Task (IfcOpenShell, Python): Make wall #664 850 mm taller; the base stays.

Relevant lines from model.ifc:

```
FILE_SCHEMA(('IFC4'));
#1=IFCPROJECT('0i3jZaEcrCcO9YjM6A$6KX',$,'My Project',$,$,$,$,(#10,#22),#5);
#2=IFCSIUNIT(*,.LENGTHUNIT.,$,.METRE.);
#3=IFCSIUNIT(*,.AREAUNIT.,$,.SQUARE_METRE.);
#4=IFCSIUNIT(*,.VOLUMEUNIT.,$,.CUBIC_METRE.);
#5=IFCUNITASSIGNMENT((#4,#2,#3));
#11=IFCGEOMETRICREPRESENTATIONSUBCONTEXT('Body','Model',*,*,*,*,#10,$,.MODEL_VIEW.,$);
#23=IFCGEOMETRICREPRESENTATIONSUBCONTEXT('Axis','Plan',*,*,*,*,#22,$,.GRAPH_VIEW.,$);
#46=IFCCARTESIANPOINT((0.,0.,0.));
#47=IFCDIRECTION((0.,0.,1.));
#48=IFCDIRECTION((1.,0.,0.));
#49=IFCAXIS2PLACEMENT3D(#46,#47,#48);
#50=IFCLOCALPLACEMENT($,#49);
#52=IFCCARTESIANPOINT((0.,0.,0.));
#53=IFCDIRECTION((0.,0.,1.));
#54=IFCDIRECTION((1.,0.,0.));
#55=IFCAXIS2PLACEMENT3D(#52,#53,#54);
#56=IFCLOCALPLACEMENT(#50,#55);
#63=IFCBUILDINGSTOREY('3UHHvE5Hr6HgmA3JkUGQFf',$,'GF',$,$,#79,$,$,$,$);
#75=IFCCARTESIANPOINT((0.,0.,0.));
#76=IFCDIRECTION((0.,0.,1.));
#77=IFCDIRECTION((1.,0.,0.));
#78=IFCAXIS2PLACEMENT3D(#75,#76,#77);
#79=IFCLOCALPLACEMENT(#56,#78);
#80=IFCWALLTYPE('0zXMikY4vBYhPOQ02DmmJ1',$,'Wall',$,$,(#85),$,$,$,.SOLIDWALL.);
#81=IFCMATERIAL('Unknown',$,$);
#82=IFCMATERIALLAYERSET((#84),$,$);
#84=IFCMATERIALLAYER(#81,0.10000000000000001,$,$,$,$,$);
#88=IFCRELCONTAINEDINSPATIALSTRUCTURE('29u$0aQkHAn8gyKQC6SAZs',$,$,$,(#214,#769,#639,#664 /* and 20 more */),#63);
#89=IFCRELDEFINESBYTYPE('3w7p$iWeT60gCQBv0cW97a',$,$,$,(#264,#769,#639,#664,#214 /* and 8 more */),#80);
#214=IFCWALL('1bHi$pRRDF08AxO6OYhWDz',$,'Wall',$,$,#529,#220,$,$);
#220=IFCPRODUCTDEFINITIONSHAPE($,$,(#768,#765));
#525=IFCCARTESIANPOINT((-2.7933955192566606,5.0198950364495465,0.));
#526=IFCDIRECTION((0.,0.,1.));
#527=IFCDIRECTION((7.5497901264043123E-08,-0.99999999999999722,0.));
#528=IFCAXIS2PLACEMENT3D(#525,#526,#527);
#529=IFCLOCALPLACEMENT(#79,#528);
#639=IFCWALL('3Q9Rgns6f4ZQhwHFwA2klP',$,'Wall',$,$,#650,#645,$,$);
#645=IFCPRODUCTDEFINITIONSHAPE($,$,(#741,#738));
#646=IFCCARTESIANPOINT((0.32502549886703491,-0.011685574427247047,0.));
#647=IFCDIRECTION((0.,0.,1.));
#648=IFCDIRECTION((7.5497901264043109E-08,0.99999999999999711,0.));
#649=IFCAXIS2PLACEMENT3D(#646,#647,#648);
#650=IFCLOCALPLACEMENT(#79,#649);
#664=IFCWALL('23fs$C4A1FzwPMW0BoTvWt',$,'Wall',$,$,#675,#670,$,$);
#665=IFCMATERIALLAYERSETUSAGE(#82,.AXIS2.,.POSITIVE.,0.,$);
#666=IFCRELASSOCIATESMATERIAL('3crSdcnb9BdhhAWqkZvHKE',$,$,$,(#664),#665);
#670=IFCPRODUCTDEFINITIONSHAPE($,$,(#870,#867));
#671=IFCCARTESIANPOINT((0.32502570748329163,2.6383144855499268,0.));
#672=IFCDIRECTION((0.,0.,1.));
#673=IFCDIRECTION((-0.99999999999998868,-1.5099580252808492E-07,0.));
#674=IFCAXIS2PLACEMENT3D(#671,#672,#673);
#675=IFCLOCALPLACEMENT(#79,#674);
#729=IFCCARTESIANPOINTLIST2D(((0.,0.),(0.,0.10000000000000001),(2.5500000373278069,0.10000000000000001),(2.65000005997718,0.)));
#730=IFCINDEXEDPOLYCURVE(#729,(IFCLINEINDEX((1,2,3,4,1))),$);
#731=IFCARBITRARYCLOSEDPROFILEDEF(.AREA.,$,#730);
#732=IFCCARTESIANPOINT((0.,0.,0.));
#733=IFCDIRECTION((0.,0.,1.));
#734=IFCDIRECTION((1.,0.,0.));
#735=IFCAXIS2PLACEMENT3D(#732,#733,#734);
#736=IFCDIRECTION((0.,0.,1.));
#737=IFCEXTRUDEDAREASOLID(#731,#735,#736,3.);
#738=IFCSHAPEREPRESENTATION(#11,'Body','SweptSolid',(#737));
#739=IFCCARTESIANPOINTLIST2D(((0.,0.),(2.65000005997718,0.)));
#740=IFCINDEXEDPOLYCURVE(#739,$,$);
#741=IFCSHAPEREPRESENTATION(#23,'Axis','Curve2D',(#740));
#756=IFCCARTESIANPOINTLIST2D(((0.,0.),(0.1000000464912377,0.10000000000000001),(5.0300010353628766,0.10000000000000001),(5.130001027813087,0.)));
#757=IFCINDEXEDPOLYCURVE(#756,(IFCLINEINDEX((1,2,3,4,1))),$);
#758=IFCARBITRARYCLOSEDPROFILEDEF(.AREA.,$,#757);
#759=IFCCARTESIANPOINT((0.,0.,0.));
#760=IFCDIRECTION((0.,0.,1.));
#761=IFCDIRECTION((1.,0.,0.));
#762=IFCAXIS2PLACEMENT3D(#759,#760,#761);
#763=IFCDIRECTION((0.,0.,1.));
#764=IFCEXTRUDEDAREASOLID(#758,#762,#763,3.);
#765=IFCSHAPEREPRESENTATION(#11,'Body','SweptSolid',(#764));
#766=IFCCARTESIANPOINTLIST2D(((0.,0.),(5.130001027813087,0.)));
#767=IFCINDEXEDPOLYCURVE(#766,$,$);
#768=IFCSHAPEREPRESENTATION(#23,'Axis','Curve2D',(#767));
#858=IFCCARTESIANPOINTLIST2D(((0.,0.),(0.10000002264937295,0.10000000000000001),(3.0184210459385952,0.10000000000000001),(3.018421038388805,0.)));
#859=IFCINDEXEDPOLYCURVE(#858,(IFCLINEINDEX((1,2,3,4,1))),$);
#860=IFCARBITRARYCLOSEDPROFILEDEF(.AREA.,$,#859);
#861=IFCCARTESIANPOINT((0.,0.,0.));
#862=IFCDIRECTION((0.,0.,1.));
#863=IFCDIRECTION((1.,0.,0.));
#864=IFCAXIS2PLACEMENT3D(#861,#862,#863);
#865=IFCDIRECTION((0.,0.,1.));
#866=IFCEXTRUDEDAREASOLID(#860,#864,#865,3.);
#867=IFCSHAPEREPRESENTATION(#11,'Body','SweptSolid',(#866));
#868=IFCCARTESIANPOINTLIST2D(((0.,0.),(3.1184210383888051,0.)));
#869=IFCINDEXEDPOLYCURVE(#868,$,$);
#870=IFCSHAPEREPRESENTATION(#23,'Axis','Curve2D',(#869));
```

```python
import ifcopenshell
import ifcopenshell.geom
import ifcopenshell.util.representation
import ifcopenshell.util.shape
import ifcopenshell.util.unit

model = ifcopenshell.open("model.ifc")
unit_scale = ifcopenshell.util.unit.calculate_unit_scale(model)
settings = ifcopenshell.geom.settings()


def volume(element):
    """Net volume in cubic metres, openings subtracted."""
    shape = ifcopenshell.geom.create_shape(settings, element)
    return ifcopenshell.util.shape.get_volume(shape.geometry)


wall = model.by_guid("23fs$C4A1FzwPMW0BoTvWt")
before = volume(wall)

body = ifcopenshell.util.representation.get_representation(wall, "Model", "Body")
solid = body.Items[0]
old_height = solid.Depth
solid.Depth += 0.85 / unit_scale
after = volume(wall)

print(f"height {old_height:g} -> {solid.Depth:g}, volume {before:.3f} -> {after:.3f} m3")

model.write("model_rev.ifc")
```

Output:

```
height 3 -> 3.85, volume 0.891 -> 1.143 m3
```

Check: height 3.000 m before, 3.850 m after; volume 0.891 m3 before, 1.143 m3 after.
